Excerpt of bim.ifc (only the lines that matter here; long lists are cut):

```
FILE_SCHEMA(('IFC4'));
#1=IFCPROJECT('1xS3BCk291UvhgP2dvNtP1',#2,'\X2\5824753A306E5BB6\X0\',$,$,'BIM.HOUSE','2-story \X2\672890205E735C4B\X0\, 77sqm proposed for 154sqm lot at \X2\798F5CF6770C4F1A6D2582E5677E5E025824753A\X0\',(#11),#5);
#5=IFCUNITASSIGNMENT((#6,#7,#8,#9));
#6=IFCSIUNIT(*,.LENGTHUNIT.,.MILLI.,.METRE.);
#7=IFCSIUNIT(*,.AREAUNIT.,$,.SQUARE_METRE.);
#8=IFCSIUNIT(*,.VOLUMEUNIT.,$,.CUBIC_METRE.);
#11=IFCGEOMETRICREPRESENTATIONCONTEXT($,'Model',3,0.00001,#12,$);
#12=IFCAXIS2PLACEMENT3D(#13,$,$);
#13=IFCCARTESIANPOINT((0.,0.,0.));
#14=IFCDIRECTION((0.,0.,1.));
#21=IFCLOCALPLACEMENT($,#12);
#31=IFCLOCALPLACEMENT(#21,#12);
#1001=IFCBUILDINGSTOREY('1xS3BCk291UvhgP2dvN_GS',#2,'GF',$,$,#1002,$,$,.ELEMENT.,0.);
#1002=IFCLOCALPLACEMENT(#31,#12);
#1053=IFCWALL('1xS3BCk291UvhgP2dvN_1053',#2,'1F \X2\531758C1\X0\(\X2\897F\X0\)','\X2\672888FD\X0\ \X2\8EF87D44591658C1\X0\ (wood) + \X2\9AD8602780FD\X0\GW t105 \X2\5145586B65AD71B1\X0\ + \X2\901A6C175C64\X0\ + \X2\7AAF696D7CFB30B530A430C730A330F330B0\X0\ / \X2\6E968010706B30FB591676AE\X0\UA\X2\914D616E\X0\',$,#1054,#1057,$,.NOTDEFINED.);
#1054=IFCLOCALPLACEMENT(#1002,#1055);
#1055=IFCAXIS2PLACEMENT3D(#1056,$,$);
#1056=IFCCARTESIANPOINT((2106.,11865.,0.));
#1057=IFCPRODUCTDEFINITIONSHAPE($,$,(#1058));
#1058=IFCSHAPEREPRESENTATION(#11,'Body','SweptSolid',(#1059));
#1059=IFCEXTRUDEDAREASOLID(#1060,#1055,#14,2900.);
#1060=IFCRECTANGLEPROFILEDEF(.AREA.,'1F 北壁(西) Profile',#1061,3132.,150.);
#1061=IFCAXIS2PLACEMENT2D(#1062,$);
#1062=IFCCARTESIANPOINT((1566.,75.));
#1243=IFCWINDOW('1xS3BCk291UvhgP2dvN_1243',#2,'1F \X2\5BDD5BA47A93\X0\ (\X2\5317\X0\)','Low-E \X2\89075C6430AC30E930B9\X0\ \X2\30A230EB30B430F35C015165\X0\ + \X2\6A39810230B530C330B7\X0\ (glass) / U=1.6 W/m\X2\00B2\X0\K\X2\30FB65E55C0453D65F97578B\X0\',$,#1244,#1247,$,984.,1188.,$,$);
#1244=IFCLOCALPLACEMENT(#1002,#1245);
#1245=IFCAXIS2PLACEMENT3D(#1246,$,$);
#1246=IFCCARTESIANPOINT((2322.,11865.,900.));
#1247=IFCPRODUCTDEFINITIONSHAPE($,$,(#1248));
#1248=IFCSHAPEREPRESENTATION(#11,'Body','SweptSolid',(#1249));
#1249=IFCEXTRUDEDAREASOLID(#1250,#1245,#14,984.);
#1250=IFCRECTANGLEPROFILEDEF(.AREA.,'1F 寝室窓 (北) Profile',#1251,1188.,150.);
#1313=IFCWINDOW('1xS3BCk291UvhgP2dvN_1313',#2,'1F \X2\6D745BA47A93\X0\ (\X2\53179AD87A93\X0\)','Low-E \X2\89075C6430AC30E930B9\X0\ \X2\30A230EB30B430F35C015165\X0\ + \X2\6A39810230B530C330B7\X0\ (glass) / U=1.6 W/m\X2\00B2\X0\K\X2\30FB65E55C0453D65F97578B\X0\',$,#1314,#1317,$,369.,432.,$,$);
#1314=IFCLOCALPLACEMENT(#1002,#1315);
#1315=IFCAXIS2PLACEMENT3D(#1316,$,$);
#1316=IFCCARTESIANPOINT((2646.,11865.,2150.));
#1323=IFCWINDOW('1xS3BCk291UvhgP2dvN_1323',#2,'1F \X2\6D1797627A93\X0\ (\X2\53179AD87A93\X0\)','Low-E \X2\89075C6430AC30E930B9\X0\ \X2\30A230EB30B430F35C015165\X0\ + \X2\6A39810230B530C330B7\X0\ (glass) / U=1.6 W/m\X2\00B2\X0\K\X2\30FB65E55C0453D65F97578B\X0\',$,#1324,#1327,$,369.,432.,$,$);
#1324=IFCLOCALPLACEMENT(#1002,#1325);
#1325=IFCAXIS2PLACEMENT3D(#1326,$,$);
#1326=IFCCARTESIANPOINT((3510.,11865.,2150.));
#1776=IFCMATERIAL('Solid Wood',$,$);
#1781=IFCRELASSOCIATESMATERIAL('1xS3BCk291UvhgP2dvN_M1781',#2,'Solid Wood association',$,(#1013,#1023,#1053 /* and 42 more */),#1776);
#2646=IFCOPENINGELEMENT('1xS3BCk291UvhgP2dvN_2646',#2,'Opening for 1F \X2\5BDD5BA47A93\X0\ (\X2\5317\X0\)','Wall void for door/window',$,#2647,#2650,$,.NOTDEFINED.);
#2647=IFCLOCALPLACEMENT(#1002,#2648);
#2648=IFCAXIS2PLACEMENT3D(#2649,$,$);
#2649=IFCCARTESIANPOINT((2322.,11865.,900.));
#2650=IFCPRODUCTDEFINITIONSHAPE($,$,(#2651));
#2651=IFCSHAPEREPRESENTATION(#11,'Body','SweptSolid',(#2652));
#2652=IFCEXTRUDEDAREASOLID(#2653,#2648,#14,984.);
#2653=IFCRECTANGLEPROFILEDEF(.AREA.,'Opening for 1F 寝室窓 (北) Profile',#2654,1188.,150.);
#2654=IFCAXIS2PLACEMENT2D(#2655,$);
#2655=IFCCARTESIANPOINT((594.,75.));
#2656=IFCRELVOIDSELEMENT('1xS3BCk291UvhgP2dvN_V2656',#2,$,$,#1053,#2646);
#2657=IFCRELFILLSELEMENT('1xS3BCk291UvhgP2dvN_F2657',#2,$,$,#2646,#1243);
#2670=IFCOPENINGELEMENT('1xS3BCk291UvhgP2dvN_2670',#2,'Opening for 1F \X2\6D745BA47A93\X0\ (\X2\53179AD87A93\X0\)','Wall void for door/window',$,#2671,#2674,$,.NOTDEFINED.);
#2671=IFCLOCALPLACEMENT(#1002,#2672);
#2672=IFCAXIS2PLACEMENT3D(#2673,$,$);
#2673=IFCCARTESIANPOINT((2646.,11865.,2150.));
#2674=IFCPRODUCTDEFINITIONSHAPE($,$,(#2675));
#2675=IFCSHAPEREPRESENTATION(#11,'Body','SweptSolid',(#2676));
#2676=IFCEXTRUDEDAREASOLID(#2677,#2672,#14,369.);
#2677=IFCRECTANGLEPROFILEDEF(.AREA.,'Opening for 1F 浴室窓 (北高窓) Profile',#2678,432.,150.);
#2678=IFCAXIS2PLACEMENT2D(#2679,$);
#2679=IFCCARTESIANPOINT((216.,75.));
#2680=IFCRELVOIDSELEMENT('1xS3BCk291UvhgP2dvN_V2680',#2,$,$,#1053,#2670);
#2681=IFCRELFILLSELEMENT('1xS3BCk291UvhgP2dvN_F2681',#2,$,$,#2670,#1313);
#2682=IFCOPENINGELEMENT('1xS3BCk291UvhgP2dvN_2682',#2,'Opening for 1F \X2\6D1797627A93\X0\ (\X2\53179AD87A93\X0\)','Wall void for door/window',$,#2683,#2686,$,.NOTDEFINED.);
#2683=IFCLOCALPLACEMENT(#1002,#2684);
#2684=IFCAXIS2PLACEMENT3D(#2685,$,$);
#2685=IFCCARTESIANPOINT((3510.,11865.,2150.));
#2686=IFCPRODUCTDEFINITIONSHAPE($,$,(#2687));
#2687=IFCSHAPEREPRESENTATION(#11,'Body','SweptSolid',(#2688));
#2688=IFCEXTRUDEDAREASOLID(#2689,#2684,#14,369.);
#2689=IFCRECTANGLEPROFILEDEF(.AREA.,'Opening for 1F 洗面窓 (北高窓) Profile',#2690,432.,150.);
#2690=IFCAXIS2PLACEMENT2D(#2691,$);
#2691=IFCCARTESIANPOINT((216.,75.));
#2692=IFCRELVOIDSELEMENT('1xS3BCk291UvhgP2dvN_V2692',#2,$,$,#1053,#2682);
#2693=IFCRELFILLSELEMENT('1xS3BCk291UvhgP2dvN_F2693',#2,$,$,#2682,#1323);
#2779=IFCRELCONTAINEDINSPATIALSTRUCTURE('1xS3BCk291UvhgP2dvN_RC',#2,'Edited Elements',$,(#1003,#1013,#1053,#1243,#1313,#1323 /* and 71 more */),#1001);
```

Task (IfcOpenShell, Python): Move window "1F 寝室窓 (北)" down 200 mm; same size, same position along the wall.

```python
import numpy as np
import ifcopenshell
import ifcopenshell.api.geometry
import ifcopenshell.util.placement
import ifcopenshell.util.unit

model = ifcopenshell.open("bim.ifc")
unit_scale = ifcopenshell.util.unit.calculate_unit_scale(model)

window = model.by_guid("1xS3BCk291UvhgP2dvN_1243")
opening = window.FillsVoids[0].RelatingOpeningElement
dz = -200.0

shift = np.array([0.0, 0.0, dz])
# The window is not placed relative to its opening, so move both.
for product in (opening, window):
    matrix = ifcopenshell.util.placement.get_local_placement(product.ObjectPlacement)
    matrix[:3, 3] += shift
    ifcopenshell.api.geometry.edit_object_placement(model, product=product, matrix=matrix, is_si=False)

print(f"moved by {dz * unit_scale:+.3f} m")

model.write("bim-out.ifc")
```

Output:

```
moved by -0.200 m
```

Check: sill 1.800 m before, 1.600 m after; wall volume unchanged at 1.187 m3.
